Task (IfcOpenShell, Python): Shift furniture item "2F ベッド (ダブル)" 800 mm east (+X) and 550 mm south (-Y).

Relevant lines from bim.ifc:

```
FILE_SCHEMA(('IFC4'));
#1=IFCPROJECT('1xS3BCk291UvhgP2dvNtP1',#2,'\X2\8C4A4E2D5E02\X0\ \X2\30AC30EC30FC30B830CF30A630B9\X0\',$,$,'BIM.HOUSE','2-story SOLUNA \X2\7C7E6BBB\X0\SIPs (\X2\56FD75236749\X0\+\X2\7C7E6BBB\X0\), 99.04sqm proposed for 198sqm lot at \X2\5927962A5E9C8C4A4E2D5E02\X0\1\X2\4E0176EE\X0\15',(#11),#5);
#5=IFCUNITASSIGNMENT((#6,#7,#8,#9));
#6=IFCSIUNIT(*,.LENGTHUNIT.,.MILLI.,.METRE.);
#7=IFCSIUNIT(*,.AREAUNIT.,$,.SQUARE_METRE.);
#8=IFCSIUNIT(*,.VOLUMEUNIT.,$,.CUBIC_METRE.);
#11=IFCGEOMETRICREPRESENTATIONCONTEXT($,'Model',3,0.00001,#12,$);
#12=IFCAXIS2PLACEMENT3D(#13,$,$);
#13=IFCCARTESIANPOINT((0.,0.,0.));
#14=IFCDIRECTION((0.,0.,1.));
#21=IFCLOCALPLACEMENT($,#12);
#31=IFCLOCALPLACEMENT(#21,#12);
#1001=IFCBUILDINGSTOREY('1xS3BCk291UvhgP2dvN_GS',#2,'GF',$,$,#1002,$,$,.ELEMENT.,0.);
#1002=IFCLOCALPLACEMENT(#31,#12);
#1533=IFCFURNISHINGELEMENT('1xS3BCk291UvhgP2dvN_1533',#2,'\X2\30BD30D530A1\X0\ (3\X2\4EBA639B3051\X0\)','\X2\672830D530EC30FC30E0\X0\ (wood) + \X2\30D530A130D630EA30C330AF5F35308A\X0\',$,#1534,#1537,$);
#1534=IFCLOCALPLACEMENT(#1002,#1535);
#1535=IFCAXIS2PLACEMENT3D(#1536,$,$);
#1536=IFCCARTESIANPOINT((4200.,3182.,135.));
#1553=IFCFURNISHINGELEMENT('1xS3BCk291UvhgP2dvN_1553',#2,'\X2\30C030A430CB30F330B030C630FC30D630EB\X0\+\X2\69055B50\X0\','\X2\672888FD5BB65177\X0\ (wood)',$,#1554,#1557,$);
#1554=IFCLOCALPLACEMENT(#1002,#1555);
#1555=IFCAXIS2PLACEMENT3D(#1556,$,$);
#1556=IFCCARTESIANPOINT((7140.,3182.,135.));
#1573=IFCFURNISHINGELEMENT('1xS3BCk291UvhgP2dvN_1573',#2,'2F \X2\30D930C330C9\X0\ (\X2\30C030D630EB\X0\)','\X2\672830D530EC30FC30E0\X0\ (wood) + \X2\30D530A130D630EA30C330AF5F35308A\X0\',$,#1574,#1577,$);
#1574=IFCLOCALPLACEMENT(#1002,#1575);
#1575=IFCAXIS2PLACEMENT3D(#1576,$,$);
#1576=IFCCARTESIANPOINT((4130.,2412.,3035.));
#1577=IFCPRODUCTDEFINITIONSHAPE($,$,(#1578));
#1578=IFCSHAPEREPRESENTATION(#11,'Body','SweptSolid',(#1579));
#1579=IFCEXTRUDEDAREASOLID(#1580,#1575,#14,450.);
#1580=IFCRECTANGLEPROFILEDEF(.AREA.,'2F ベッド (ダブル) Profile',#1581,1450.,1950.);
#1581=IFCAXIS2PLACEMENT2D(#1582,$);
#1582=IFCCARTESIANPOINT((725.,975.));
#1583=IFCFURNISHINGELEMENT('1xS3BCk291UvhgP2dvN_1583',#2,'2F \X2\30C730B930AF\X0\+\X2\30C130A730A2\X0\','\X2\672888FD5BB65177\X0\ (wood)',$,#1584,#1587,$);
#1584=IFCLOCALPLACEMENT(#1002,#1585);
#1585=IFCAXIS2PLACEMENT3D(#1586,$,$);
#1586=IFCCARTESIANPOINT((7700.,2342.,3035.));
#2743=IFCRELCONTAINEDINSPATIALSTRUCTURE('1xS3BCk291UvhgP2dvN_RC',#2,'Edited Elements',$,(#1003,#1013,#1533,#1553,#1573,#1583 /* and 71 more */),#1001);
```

```python
import ifcopenshell
import ifcopenshell.api.geometry
import ifcopenshell.util.placement
import ifcopenshell.util.unit

model = ifcopenshell.open("bim.ifc")
unit_scale = ifcopenshell.util.unit.calculate_unit_scale(model)

item = model.by_guid("1xS3BCk291UvhgP2dvN_1573")
matrix = ifcopenshell.util.placement.get_local_placement(item.ObjectPlacement)
matrix[0, 3] += 0.8 / unit_scale
matrix[1, 3] -= 0.55 / unit_scale
ifcopenshell.api.geometry.edit_object_placement(model, product=item, matrix=matrix, is_si=False)

print(ifcopenshell.util.placement.get_local_placement(item.ObjectPlacement).round(3) + 0.0)

model.write("bim-out.ifc")
```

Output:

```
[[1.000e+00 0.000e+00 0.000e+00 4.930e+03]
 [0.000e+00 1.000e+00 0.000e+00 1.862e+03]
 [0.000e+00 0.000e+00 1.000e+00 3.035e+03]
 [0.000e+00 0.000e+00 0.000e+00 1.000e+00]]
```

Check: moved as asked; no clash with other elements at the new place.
